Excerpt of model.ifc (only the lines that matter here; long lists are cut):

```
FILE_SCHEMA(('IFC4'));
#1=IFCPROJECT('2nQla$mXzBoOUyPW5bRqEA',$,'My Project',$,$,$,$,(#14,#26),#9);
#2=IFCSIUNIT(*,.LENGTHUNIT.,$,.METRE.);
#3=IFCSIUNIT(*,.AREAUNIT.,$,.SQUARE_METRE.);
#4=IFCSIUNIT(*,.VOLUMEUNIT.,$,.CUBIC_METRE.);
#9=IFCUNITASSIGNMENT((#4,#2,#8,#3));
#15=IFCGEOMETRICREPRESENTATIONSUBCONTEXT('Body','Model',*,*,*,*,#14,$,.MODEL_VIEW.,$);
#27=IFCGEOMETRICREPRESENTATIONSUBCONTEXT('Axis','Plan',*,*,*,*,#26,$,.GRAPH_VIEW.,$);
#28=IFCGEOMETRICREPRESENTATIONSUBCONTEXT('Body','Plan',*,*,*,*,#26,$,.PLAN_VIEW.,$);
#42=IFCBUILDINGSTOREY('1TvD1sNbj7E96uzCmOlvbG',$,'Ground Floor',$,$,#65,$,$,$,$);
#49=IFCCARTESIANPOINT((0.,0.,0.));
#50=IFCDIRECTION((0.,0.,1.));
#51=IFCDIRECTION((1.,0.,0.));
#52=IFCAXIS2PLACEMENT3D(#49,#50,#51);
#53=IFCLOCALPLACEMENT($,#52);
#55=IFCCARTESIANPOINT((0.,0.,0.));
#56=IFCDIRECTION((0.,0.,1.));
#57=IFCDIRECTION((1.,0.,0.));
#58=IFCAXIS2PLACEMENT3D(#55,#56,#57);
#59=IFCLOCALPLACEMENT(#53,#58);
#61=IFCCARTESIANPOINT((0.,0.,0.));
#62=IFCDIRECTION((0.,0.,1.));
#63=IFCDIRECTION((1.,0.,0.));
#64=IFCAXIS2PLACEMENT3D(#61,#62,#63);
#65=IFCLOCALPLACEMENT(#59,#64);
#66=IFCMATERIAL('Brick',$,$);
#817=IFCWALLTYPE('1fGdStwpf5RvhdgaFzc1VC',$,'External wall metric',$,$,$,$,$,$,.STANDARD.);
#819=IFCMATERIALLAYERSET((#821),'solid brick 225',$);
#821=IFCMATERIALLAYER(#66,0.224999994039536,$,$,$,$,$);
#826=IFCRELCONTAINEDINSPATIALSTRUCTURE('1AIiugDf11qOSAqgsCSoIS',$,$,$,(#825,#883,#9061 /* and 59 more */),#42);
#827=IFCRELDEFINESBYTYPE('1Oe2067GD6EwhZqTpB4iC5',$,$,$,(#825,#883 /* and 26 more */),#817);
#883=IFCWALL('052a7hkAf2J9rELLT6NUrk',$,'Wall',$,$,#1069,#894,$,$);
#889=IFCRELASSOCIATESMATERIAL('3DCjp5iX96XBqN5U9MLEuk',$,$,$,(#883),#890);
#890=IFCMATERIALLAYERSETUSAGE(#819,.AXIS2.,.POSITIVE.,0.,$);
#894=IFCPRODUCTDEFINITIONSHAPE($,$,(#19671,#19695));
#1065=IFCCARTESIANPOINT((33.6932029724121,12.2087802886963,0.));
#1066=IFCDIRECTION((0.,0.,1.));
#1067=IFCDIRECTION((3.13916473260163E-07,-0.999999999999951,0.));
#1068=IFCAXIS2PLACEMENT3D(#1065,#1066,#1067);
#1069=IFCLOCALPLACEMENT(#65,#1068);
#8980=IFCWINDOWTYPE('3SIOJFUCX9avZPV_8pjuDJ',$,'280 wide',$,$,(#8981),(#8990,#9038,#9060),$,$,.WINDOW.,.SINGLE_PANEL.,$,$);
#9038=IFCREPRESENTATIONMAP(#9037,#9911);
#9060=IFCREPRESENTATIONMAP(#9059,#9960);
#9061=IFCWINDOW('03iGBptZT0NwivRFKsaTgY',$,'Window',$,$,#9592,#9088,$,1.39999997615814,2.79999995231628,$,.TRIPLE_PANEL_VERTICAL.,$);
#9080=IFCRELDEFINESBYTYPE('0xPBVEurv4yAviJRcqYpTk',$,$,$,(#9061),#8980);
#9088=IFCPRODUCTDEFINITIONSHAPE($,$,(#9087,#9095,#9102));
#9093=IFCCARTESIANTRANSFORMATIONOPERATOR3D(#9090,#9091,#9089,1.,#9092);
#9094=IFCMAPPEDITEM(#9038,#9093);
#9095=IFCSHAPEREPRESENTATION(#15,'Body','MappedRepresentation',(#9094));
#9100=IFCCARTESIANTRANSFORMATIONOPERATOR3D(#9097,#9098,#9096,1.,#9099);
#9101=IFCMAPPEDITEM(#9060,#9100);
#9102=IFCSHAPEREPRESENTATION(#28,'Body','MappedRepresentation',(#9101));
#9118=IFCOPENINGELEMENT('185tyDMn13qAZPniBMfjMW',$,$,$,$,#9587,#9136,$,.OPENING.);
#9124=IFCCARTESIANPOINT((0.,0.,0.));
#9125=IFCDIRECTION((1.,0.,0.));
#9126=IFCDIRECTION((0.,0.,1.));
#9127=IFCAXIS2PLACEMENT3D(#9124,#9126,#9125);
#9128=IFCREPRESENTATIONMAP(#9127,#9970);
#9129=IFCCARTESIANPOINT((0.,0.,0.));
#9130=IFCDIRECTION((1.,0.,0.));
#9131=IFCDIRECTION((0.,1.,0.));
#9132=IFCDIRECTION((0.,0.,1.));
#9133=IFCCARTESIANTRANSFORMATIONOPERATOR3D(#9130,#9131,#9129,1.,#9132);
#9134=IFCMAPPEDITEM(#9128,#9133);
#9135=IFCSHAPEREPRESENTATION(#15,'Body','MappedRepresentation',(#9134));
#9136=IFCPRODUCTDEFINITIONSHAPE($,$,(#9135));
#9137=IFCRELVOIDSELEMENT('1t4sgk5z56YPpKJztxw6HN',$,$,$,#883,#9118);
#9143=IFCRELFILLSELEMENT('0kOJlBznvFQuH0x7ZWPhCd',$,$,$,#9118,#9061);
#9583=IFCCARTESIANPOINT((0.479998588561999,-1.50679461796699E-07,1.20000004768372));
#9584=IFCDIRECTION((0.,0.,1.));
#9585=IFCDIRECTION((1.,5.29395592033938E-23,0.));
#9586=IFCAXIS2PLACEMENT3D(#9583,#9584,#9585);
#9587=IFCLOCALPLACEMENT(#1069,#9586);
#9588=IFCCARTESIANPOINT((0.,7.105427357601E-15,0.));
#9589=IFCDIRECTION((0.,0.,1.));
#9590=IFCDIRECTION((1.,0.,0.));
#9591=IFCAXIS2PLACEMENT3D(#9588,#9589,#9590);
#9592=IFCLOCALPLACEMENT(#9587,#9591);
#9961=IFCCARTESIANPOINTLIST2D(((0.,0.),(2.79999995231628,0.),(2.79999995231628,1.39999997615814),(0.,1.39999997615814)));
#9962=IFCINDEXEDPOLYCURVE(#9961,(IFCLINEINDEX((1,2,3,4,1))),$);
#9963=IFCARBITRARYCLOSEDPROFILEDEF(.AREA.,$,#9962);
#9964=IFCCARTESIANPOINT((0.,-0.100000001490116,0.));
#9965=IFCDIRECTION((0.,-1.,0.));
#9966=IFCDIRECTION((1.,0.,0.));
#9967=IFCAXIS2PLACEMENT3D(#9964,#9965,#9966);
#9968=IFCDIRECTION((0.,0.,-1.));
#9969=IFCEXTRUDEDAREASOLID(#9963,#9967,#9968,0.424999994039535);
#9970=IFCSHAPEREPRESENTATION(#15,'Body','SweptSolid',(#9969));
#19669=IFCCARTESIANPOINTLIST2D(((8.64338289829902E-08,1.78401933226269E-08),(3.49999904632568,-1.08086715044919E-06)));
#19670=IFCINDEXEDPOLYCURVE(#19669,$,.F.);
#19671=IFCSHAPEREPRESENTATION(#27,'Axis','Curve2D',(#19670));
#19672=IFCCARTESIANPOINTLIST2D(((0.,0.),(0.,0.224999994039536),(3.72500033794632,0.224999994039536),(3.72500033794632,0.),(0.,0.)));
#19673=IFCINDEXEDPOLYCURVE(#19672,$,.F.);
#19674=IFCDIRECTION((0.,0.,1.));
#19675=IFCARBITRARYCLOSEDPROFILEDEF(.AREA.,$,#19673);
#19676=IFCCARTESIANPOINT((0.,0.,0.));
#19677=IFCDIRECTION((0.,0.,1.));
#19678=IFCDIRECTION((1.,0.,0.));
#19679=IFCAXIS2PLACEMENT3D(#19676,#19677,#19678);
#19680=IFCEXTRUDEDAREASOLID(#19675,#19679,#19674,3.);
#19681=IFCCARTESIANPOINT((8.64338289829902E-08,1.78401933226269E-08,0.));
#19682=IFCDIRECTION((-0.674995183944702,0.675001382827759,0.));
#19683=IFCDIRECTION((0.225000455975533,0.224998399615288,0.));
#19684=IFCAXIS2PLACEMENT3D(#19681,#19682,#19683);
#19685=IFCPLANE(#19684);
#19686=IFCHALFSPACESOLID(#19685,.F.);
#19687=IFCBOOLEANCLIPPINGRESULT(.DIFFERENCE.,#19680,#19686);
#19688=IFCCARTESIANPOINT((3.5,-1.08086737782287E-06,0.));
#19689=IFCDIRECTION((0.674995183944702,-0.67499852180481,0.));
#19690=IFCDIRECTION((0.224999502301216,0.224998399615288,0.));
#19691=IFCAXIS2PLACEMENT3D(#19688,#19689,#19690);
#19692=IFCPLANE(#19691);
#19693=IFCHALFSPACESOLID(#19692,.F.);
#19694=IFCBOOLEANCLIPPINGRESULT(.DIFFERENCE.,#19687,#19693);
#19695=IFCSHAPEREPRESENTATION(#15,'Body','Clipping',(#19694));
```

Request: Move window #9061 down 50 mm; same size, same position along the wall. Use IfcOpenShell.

```python
import numpy as np
import ifcopenshell
import ifcopenshell.api.geometry
import ifcopenshell.util.placement
import ifcopenshell.util.unit

model = ifcopenshell.open("model.ifc")
unit_scale = ifcopenshell.util.unit.calculate_unit_scale(model)

window = model.by_id(9061)
opening = window.FillsVoids[0].RelatingOpeningElement
dz = -0.05 / unit_scale

shift = np.array([0.0, 0.0, dz])
# The window is placed relative to its opening, so it follows when the opening moves.
matrix = ifcopenshell.util.placement.get_local_placement(opening.ObjectPlacement)
matrix[:3, 3] += shift
ifcopenshell.api.geometry.edit_object_placement(
    model, product=opening, matrix=matrix, is_si=False, should_transform_children=True
)

print(f"moved by {dz * unit_scale:+.3f} m")

model.write("model_rev.ifc")
```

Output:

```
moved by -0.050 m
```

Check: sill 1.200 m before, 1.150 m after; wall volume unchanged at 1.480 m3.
